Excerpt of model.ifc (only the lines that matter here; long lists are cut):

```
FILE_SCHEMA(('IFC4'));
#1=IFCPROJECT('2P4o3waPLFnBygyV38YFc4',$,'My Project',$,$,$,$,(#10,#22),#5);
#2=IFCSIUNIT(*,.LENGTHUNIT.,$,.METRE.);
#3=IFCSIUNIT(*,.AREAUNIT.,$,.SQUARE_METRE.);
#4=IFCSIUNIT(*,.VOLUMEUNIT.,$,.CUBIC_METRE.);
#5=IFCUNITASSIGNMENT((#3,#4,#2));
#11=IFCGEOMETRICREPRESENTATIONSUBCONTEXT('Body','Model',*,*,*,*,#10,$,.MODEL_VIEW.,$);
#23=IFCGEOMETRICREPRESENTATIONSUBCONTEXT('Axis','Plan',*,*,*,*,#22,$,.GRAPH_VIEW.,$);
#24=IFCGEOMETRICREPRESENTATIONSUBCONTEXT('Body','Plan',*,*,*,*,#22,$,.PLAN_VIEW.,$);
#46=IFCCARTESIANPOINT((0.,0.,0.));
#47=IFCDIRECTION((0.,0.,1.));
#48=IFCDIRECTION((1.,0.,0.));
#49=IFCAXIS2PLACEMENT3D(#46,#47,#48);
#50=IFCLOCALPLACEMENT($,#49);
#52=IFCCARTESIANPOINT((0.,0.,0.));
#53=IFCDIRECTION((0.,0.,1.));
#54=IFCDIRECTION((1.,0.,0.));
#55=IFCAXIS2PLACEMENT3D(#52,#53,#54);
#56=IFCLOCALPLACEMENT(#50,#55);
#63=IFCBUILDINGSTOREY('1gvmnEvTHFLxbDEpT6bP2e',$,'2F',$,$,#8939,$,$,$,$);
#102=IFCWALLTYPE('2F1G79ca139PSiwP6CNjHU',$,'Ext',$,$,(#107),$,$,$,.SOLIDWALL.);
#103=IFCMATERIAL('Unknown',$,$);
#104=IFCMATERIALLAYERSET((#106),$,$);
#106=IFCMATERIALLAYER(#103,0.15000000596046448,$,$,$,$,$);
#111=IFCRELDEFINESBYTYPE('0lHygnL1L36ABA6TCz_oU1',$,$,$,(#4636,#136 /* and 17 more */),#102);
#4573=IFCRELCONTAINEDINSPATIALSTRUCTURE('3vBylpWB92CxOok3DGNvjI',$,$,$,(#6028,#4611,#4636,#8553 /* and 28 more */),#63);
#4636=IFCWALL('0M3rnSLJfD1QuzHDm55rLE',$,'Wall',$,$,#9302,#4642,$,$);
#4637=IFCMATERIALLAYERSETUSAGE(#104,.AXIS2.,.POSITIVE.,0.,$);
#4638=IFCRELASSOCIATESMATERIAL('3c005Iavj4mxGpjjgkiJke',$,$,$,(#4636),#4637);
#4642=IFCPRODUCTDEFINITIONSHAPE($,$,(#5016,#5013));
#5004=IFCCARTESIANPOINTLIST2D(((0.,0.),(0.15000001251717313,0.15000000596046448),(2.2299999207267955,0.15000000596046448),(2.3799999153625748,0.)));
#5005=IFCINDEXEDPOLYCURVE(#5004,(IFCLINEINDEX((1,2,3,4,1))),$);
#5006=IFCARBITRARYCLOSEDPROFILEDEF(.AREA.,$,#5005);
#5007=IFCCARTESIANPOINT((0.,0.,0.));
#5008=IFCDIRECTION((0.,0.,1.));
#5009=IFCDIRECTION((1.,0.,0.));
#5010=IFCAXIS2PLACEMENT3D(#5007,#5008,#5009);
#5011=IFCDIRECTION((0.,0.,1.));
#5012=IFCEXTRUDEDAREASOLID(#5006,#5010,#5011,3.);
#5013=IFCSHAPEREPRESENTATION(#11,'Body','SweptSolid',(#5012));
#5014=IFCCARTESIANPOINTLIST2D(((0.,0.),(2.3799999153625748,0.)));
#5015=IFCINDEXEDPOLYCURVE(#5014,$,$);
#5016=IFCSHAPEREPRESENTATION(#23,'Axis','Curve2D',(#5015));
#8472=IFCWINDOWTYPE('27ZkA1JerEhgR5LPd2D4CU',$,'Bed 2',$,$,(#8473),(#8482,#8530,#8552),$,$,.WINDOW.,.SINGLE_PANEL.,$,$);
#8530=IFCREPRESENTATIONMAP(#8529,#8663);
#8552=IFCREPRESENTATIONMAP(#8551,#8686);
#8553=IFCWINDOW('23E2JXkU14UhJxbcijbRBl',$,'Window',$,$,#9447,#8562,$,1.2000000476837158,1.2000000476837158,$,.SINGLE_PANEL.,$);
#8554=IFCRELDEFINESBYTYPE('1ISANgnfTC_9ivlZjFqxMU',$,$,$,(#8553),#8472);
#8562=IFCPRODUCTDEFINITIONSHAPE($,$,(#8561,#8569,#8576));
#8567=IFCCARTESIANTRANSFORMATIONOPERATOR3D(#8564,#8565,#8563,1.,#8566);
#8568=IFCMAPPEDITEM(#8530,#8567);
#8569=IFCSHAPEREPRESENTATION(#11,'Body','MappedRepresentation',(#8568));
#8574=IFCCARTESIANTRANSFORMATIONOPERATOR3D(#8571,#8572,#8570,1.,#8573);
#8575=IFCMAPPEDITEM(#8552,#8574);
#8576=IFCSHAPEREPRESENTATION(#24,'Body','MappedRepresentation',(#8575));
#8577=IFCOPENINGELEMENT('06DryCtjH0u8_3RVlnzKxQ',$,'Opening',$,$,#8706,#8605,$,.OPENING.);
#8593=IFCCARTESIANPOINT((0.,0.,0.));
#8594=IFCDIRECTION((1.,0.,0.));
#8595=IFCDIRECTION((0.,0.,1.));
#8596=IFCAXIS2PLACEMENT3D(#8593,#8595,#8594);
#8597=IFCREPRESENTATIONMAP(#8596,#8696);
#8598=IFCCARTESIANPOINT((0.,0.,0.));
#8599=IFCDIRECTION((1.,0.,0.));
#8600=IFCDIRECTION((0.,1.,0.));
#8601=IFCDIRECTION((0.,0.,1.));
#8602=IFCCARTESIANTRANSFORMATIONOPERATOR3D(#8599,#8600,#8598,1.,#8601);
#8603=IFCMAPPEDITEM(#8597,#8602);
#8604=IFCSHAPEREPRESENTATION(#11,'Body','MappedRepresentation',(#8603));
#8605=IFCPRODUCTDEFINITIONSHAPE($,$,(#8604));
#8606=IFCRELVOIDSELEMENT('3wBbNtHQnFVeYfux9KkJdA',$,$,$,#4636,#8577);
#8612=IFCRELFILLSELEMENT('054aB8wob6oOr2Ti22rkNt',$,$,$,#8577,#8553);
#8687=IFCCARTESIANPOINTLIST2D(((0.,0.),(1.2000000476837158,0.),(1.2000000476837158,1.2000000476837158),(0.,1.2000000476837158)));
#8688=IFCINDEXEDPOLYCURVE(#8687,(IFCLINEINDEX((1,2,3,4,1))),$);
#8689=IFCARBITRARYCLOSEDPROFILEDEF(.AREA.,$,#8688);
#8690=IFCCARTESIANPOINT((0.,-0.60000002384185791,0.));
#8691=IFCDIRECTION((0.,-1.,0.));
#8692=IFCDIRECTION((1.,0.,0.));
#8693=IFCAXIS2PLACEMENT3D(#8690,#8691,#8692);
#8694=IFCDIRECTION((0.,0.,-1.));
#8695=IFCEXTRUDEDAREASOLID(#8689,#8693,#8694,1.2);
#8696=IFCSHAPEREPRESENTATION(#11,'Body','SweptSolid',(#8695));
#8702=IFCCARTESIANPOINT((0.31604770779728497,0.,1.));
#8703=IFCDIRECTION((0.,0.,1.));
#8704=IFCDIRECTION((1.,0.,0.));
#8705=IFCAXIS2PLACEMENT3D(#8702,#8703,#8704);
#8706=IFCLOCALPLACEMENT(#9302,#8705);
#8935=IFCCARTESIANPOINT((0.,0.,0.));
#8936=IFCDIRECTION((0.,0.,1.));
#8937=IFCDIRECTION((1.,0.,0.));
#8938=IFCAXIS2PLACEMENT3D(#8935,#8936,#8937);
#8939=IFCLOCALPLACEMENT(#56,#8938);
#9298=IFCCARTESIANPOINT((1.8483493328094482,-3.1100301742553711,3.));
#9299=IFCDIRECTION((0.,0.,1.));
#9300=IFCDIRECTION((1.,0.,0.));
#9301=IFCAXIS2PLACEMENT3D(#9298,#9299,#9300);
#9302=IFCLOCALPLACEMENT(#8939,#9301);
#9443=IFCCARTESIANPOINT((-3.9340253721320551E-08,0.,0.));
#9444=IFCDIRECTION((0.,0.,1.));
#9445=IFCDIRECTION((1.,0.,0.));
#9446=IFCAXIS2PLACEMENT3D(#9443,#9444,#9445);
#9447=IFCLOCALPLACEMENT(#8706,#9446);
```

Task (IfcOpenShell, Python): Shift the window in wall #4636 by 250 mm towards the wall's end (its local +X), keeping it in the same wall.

```python
import ifcopenshell
import ifcopenshell.api.geometry
import ifcopenshell.util.placement

model = ifcopenshell.open("model.ifc")

window = model.by_guid("23E2JXkU14UhJxbcijbRBl")
opening = window.FillsVoids[0].RelatingOpeningElement
wall = opening.VoidsElements[0].RelatingBuildingElement

wall_matrix = ifcopenshell.util.placement.get_local_placement(wall.ObjectPlacement)
shift = wall_matrix[:3, 0] * 0.25
before = ifcopenshell.util.placement.get_local_placement(window.ObjectPlacement)[:3, 3].copy()

# The window is placed relative to its opening, so it follows when the opening moves.
matrix = ifcopenshell.util.placement.get_local_placement(opening.ObjectPlacement)
matrix[:3, 3] += shift
ifcopenshell.api.geometry.edit_object_placement(
    model, product=opening, matrix=matrix, is_si=False, should_transform_children=True
)

after = ifcopenshell.util.placement.get_local_placement(window.ObjectPlacement)[:3, 3]
print("window moved by", (after - before).round(3) + 0.0)

model.write("model-out.ifc")
```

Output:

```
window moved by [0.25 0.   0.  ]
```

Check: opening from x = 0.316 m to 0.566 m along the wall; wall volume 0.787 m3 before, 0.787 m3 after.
